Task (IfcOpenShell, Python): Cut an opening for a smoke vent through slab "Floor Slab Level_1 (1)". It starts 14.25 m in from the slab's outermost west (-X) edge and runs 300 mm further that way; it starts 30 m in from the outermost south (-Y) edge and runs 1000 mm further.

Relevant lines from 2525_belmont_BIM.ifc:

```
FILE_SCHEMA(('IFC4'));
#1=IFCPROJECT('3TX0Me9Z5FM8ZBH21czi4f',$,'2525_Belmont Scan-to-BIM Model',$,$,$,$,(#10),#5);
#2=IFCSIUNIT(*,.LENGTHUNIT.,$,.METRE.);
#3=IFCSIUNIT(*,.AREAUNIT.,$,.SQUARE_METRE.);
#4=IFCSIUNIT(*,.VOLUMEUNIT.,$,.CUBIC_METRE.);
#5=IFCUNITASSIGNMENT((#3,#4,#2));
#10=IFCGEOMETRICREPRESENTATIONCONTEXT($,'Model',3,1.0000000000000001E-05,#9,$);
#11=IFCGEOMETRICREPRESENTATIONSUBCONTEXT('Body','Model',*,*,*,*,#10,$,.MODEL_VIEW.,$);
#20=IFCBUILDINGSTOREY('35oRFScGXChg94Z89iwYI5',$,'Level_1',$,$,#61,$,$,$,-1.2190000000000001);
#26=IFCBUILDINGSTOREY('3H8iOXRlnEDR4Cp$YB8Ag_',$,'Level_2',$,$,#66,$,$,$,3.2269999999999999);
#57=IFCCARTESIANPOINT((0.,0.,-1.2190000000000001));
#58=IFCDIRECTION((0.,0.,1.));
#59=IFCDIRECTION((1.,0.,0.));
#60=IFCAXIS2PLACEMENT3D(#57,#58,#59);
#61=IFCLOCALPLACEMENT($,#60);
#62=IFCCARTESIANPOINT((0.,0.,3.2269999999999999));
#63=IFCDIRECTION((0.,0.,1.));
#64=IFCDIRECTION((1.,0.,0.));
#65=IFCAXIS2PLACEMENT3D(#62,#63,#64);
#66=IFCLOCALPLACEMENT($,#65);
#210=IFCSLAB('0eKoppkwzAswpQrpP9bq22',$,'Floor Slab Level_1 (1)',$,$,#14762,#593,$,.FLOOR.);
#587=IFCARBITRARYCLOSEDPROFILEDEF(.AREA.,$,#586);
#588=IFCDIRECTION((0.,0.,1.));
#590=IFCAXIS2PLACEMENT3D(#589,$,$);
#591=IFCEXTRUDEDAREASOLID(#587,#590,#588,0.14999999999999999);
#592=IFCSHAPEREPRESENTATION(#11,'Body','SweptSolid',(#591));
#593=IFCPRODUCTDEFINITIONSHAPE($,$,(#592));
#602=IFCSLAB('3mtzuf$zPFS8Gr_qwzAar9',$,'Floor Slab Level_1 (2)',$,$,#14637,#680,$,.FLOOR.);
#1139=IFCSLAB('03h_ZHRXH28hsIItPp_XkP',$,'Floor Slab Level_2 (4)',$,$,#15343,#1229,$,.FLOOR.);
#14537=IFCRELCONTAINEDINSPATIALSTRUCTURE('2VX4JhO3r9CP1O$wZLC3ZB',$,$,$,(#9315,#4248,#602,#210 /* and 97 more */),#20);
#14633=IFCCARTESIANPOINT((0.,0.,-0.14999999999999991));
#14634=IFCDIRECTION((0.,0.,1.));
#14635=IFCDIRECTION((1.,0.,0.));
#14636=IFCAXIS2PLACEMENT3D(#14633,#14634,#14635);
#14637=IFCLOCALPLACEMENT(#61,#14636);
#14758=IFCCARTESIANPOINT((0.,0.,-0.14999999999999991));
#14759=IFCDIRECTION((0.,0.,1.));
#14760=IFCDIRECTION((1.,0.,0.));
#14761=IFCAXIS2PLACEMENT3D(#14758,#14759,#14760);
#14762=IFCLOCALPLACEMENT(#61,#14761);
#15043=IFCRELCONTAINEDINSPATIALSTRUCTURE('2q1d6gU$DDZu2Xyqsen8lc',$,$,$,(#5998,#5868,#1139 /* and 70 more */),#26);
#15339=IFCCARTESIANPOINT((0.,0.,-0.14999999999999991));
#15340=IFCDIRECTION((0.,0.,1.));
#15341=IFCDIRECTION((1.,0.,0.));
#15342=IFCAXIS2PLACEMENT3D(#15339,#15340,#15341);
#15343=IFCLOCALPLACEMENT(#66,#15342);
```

```python
import numpy as np
import ifcopenshell
import ifcopenshell.api.feature
import ifcopenshell.api.geometry
import ifcopenshell.api.root
import ifcopenshell.geom
import ifcopenshell.util.placement
import ifcopenshell.util.representation
import ifcopenshell.util.shape
import ifcopenshell.util.unit

model = ifcopenshell.open("2525_belmont_BIM.ifc")
unit_scale = ifcopenshell.util.unit.calculate_unit_scale(model)
settings = ifcopenshell.geom.settings()


def volume(element):
    """Net volume in cubic metres, openings subtracted."""
    shape = ifcopenshell.geom.create_shape(settings, element)
    return ifcopenshell.util.shape.get_volume(shape.geometry)


slab = model.by_guid("0eKoppkwzAswpQrpP9bq22")
before = volume(slab)

# Extent in the slab's own axes, in metres. The edges named are its -X and -Y sides.
slab_shape = ifcopenshell.geom.create_shape(settings, slab)
vertices = ifcopenshell.util.shape.get_vertices(slab_shape.geometry)
x_min, y_min, bottom = vertices.min(axis=0)
top = vertices[:, 2].max()

opening = ifcopenshell.api.root.create_entity(model, ifc_class="IfcOpeningElement", name="Smoke vent opening", predefined_type="OPENING")
context = ifcopenshell.util.representation.get_context(model, "Model", "Body", "MODEL_VIEW")
width, depth = 0.3, 1
outline = [(0.0, 0.0), (width, 0.0), (width, depth), (0.0, depth), (0.0, 0.0)]
# Overshoot both faces by 50 mm so the cut is clean.
shape = ifcopenshell.api.geometry.add_slab_representation(
    model, context=context, depth=top - bottom + 0.1, polyline=outline
)
ifcopenshell.api.geometry.assign_representation(model, product=opening, representation=shape)

matrix = ifcopenshell.util.placement.get_local_placement(slab.ObjectPlacement)
matrix[:, 3] = matrix @ np.append(np.array([x_min + 14.25, y_min + 30, bottom - 0.05]) / unit_scale, 1.0)
ifcopenshell.api.geometry.edit_object_placement(model, product=opening, matrix=matrix, is_si=False)
ifcopenshell.api.feature.add_feature(model, feature=opening, element=slab)

after = volume(slab)

print(f"slab volume {before:.3f} -> {after:.3f} m3")

model.write("2525_belmont_BIM-out.ifc")
```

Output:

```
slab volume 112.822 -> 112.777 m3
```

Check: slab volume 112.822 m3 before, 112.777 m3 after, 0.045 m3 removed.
